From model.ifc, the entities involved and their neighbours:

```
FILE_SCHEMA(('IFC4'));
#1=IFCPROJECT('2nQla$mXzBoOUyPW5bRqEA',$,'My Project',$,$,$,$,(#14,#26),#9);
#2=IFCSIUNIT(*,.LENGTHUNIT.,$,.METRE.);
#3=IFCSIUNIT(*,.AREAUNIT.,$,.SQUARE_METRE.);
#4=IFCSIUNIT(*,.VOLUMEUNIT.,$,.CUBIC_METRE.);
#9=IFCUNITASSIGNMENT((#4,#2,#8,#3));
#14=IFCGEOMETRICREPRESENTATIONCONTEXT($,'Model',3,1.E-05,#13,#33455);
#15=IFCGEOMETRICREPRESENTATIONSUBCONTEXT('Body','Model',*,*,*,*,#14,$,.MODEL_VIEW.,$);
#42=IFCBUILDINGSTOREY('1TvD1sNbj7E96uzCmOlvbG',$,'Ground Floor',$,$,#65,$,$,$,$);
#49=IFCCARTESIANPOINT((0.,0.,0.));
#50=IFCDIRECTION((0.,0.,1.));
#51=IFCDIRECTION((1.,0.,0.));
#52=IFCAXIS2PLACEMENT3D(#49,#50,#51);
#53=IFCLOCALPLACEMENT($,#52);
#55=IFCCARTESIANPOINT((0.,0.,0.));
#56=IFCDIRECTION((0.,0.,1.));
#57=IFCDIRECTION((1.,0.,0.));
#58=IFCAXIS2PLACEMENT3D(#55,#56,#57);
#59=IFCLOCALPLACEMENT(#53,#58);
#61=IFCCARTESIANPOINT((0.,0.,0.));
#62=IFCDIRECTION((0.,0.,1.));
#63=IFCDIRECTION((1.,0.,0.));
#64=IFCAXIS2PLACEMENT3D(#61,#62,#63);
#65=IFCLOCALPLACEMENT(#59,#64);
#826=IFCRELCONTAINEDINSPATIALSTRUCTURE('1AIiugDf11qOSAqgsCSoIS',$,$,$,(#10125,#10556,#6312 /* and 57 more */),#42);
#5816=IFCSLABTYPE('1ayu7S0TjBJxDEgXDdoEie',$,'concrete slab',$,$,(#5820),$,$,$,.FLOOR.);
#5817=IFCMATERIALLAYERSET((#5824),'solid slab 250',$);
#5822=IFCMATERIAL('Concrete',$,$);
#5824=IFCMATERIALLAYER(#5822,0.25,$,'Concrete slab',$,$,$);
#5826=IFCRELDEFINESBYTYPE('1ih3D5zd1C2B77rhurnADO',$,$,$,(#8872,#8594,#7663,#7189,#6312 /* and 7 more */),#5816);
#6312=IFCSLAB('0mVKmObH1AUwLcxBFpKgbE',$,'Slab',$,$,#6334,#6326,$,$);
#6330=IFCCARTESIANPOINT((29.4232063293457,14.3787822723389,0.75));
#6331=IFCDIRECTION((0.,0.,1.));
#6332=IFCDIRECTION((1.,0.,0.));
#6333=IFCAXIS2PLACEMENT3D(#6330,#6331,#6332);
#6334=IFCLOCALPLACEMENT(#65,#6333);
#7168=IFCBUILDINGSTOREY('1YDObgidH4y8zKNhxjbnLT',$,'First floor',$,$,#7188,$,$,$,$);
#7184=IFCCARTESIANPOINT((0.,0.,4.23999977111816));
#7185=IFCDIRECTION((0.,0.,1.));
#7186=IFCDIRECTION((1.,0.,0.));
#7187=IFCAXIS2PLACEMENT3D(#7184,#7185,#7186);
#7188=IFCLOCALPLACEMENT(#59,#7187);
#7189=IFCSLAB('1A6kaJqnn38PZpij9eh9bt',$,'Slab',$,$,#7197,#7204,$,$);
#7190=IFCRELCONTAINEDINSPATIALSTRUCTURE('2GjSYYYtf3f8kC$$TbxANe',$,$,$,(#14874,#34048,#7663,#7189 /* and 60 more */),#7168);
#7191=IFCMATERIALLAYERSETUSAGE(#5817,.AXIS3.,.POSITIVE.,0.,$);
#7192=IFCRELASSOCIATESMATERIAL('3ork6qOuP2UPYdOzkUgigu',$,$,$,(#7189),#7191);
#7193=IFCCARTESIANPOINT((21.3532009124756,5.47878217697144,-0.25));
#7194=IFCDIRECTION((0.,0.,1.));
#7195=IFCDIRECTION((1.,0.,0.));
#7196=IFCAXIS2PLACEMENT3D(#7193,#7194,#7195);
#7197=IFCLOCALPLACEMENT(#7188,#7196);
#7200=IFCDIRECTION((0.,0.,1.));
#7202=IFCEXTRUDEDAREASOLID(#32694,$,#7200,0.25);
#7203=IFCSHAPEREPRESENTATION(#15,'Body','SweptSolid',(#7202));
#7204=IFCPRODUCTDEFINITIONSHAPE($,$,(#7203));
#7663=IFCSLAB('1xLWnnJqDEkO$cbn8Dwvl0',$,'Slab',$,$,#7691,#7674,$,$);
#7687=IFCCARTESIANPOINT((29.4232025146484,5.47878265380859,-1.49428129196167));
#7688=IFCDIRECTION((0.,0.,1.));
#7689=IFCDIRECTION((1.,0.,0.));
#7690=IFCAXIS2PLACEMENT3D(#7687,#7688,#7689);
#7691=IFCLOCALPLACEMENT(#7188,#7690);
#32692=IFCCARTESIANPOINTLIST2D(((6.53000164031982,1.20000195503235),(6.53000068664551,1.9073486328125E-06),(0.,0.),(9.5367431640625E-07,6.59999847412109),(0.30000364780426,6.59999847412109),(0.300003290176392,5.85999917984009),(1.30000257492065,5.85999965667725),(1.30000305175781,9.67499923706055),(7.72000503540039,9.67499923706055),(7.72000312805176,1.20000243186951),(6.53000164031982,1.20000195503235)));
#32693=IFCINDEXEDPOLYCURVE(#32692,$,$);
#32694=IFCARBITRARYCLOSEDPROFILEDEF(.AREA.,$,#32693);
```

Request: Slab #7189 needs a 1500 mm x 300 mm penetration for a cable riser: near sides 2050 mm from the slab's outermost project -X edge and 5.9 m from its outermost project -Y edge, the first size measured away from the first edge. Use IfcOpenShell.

```python
import numpy as np
import ifcopenshell
import ifcopenshell.api.feature
import ifcopenshell.api.geometry
import ifcopenshell.api.root
import ifcopenshell.geom
import ifcopenshell.util.placement
import ifcopenshell.util.representation
import ifcopenshell.util.shape
import ifcopenshell.util.unit

model = ifcopenshell.open("model.ifc")
unit_scale = ifcopenshell.util.unit.calculate_unit_scale(model)
settings = ifcopenshell.geom.settings()


def volume(element):
    """Net volume in cubic metres, openings subtracted."""
    shape = ifcopenshell.geom.create_shape(settings, element)
    return ifcopenshell.util.shape.get_volume(shape.geometry)


slab = model.by_guid("1A6kaJqnn38PZpij9eh9bt")
before = volume(slab)

# Extent in the slab's own axes, in metres. The edges named are its -X and -Y sides.
slab_shape = ifcopenshell.geom.create_shape(settings, slab)
vertices = ifcopenshell.util.shape.get_vertices(slab_shape.geometry)
x_min, y_min, bottom = vertices.min(axis=0)
top = vertices[:, 2].max()

opening = ifcopenshell.api.root.create_entity(model, ifc_class="IfcOpeningElement", name="Cable riser opening", predefined_type="OPENING")
context = ifcopenshell.util.representation.get_context(model, "Model", "Body", "MODEL_VIEW")
width, depth = 1.5, 0.3
outline = [(0.0, 0.0), (width, 0.0), (width, depth), (0.0, depth), (0.0, 0.0)]
# Overshoot both faces by 50 mm so the cut is clean.
shape = ifcopenshell.api.geometry.add_slab_representation(
    model, context=context, depth=top - bottom + 0.1, polyline=outline
)
ifcopenshell.api.geometry.assign_representation(model, product=opening, representation=shape)

matrix = ifcopenshell.util.placement.get_local_placement(slab.ObjectPlacement)
matrix[:, 3] = matrix @ np.append(np.array([x_min + 2.05, y_min + 5.9, bottom - 0.05]) / unit_scale, 1.0)
ifcopenshell.api.geometry.edit_object_placement(model, product=opening, matrix=matrix, is_si=False)
ifcopenshell.api.feature.add_feature(model, feature=opening, element=slab)

after = volume(slab)

print(f"slab volume {before:.3f} -> {after:.3f} m3")

model.write("model_edited.ifc")
```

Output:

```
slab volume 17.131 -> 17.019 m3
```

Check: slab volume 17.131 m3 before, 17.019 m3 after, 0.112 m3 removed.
